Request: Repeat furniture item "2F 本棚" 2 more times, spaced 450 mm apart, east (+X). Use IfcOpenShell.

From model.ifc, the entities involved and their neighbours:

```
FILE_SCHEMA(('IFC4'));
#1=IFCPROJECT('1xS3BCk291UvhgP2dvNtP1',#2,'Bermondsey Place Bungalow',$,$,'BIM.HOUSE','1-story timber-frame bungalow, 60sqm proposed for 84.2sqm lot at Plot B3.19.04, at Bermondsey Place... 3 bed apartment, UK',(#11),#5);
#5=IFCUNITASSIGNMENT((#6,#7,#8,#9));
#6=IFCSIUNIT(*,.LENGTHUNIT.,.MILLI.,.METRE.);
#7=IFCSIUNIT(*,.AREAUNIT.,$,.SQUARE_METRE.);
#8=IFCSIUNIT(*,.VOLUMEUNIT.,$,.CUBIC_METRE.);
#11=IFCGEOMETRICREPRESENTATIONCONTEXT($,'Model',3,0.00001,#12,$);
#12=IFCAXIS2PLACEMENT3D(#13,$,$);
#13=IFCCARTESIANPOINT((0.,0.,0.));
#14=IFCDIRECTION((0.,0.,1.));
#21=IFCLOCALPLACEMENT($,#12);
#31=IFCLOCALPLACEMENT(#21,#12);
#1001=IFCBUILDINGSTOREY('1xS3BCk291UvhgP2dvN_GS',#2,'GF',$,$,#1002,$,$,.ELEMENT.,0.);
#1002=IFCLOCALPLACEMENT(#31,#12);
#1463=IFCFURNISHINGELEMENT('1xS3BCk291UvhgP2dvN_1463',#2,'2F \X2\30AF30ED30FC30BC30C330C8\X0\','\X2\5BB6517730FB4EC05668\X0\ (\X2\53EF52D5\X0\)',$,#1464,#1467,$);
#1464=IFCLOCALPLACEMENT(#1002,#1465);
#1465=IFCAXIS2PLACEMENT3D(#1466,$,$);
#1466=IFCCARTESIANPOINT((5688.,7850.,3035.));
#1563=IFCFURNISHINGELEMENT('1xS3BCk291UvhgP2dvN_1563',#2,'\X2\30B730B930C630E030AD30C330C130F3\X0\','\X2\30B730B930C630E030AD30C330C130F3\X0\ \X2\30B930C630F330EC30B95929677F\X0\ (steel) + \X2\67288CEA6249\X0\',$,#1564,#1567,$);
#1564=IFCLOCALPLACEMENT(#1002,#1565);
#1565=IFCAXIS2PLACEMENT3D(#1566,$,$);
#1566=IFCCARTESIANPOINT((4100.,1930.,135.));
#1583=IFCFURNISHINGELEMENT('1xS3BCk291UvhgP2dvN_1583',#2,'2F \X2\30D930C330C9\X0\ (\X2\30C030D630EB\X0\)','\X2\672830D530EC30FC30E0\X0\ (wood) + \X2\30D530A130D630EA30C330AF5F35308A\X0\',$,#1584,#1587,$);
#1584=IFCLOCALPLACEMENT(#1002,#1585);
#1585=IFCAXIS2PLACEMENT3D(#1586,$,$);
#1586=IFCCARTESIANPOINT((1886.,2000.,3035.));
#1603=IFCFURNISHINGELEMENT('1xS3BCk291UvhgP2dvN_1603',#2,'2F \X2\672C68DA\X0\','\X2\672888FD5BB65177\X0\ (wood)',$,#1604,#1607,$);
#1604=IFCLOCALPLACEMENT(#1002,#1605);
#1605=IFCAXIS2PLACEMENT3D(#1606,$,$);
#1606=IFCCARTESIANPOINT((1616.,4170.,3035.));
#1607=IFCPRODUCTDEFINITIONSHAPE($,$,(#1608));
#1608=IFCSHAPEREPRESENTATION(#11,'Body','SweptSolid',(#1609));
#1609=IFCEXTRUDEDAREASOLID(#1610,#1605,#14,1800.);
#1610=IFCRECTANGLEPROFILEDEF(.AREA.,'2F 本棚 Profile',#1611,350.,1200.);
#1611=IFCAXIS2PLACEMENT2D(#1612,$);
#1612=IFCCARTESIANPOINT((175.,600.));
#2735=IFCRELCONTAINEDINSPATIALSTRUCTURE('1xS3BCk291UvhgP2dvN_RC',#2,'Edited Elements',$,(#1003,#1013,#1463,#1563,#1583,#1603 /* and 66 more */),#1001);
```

```python
import numpy as np
import ifcopenshell
import ifcopenshell.api.geometry
import ifcopenshell.api.root
import ifcopenshell.util.element
import ifcopenshell.util.placement
import ifcopenshell.util.unit

model = ifcopenshell.open("model.ifc")
unit_scale = ifcopenshell.util.unit.calculate_unit_scale(model)


def reuse_history(source, copy):
    """copy_class also copies each property set's owner history, people and application; keep the originals."""
    for rel in copy.IsDefinedBy:
        if rel.is_a("IfcRelDefinesByProperties") and (history := rel.RelatingPropertyDefinition.OwnerHistory):
            rel.RelatingPropertyDefinition.OwnerHistory = source.OwnerHistory
            ifcopenshell.util.element.remove_deep2(model, history)


source = model.by_guid("1xS3BCk291UvhgP2dvN_1603")
base = ifcopenshell.util.placement.get_local_placement(source.ObjectPlacement)
step = np.array([1.0, 0.0, 0.0]) * 0.45 / unit_scale

for i in range(1, 3):
    copy = ifcopenshell.api.root.copy_class(model, product=source)
    copy.Representation = ifcopenshell.util.element.copy_deep(
        model, source.Representation, exclude=["IfcGeometricRepresentationContext", "IfcRepresentationMap"]
    )
    reuse_history(source, copy)
    matrix = base.copy()
    matrix[:3, 3] += i * step
    print("added at", matrix[:3, 3].round(3) + 0.0)
    ifcopenshell.api.geometry.edit_object_placement(model, product=copy, matrix=matrix, is_si=False)

model.write("model_updated.ifc")
```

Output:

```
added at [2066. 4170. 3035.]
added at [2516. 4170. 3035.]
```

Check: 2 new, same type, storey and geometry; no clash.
